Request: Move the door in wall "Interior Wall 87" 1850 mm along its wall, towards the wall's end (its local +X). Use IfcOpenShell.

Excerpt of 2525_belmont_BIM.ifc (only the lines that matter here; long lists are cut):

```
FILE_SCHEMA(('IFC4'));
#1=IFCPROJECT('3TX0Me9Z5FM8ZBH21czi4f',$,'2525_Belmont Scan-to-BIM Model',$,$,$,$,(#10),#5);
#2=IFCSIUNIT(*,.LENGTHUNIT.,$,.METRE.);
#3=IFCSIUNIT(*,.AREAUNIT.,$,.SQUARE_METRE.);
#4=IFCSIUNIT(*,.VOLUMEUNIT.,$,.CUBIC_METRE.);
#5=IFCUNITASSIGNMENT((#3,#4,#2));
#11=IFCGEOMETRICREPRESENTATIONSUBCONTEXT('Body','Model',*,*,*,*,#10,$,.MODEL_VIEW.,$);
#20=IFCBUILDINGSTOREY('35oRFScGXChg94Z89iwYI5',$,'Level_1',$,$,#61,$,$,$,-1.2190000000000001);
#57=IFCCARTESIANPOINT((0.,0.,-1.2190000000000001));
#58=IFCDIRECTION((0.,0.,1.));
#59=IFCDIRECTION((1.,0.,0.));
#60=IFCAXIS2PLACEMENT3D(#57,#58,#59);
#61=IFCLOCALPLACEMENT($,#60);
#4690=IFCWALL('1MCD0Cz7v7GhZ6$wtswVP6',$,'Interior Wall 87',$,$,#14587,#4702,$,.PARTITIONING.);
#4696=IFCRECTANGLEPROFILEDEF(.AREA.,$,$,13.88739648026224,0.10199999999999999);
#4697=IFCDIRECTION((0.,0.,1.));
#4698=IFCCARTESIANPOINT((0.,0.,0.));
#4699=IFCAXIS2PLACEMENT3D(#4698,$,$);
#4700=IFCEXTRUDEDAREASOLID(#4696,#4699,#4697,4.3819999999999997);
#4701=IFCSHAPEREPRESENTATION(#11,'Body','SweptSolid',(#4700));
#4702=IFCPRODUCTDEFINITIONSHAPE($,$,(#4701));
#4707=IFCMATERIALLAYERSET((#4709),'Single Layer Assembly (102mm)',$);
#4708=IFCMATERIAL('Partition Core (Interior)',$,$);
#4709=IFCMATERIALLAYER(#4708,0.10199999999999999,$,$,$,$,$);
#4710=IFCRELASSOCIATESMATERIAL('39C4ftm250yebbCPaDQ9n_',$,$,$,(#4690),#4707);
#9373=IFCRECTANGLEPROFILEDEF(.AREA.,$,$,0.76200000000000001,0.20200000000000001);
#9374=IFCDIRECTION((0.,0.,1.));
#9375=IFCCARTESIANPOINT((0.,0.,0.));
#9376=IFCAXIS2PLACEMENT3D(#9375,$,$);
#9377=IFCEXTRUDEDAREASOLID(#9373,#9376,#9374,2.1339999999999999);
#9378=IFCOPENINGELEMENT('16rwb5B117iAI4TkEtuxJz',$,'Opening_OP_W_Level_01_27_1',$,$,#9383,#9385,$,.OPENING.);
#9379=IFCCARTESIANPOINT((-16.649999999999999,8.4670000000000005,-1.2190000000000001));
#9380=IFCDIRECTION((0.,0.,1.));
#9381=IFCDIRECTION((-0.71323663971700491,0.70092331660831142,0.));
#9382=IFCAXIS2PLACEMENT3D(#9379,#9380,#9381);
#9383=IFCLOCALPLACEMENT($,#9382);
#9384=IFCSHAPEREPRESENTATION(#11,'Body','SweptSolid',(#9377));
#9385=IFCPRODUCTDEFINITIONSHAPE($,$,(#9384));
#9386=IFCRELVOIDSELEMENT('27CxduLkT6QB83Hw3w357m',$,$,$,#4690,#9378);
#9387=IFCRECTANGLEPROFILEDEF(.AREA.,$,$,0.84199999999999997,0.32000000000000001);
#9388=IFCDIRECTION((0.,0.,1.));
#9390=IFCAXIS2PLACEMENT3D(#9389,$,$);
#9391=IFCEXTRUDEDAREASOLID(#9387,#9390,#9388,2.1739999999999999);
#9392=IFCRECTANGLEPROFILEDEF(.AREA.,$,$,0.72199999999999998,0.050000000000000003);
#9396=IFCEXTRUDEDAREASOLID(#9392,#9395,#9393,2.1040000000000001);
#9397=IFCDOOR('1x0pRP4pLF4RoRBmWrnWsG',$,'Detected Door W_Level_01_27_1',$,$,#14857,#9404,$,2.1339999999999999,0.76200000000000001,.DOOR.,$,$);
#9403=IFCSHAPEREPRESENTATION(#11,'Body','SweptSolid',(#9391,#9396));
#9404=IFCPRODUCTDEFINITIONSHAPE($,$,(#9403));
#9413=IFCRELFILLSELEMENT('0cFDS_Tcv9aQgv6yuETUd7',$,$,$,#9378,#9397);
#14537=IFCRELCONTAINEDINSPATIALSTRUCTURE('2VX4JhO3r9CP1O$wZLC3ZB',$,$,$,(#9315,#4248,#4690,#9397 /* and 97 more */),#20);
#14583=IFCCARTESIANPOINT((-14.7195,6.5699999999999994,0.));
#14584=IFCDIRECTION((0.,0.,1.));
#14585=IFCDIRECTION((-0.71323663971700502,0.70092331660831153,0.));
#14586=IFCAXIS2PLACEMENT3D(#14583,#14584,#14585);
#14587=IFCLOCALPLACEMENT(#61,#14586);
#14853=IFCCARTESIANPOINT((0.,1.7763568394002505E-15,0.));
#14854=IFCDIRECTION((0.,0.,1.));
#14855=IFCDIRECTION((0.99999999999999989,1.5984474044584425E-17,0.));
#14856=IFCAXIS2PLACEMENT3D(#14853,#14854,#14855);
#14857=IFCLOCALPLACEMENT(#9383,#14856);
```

```python
import ifcopenshell
import ifcopenshell.api.geometry
import ifcopenshell.util.placement
import ifcopenshell.util.unit

model = ifcopenshell.open("2525_belmont_BIM.ifc")
unit_scale = ifcopenshell.util.unit.calculate_unit_scale(model)

door = model.by_id(9397)
opening = door.FillsVoids[0].RelatingOpeningElement
wall = opening.VoidsElements[0].RelatingBuildingElement

wall_matrix = ifcopenshell.util.placement.get_local_placement(wall.ObjectPlacement)
shift = wall_matrix[:3, 0] * 1.85 / unit_scale
before = ifcopenshell.util.placement.get_local_placement(door.ObjectPlacement)[:3, 3].copy()

# The door is placed relative to its opening, so it follows when the opening moves.
matrix = ifcopenshell.util.placement.get_local_placement(opening.ObjectPlacement)
matrix[:3, 3] += shift
ifcopenshell.api.geometry.edit_object_placement(
    model, product=opening, matrix=matrix, is_si=False, should_transform_children=True
)

after = ifcopenshell.util.placement.get_local_placement(door.ObjectPlacement)[:3, 3]
print("door moved by", (after - before).round(3) + 0.0)

model.write("2525_belmont_BIM_rev.ifc")
```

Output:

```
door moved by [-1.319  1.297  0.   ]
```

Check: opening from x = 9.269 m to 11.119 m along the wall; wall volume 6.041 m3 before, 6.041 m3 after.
